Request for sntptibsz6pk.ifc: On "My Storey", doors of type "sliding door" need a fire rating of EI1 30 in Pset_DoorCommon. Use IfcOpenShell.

First a look at what the model holds.

```python
import ifcopenshell
import ifcopenshell.util.element

model = ifcopenshell.open("sntptibsz6pk.ifc")
print(model.schema)
storey = next(s for s in model.by_type("IfcBuildingStorey") if s.Name == "My Storey")
doors = [e for e in ifcopenshell.util.element.get_decomposition(storey) if e.is_a("IfcDoor")]
seen = {}
for e in doors:
    element_type = ifcopenshell.util.element.get_type(e)
    key = (element_type.Name if element_type != e and element_type else None, ifcopenshell.util.element.get_pset(e, "Pset_DoorCommon", "FireRating"))
    seen[key] = seen.get(key, 0) + 1
for (name, value), count in sorted(seen.items(), key=str):
    print(count, "x", name, "|", value)
```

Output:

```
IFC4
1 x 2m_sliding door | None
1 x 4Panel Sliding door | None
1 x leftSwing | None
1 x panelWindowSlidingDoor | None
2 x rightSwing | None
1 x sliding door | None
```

```python
import ifcopenshell
import ifcopenshell.api.pset
import ifcopenshell.util.element

model = ifcopenshell.open("sntptibsz6pk.ifc")

storey = next(s for s in model.by_type("IfcBuildingStorey") if s.Name == "My Storey")
doors = [e for e in ifcopenshell.util.element.get_decomposition(storey) if e.is_a("IfcDoor")]

count = 0
for e in doors:
    element_type = ifcopenshell.util.element.get_type(e)
    if element_type in (None, e) or element_type.Name != "sliding door":
        continue
    # add_pset returns the element's existing set when there is one.
    pset = ifcopenshell.api.pset.add_pset(model, product=e, name="Pset_DoorCommon")
    ifcopenshell.api.pset.edit_pset(model, pset=pset, properties={"FireRating": "EI1 30"})
    count += 1

print(count, "doors updated")

model.write("sntptibsz6pk_updated.ifc")
```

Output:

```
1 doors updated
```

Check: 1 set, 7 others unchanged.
